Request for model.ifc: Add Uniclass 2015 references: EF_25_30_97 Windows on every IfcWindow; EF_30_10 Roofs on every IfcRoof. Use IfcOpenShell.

First a look at what the model holds.

```python
import ifcopenshell

model = ifcopenshell.open("model.ifc")
print(model.schema)
print("classifications:", [c.Name for c in model.by_type("IfcClassification")])
for ifc_class in ("IfcDoor", "IfcRoof", "IfcStair", "IfcWall", "IfcWindow"):
    print(ifc_class, len(model.by_type(ifc_class)))
```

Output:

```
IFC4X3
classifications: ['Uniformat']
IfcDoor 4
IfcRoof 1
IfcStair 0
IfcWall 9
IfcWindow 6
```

```python
import ifcopenshell
import ifcopenshell.api.classification

model = ifcopenshell.open("model.ifc")

system = ifcopenshell.api.classification.add_classification(model, classification="Uniclass 2015")

codes = {
    "IfcWindow": ("EF_25_30_97", "Windows"),
    "IfcRoof": ("EF_30_10", "Roofs"),
}
for ifc_class, (code, name) in codes.items():
    products = model.by_type(ifc_class)
    ifcopenshell.api.classification.add_reference(
        model, products=products, classification=system, identification=code, name=name
    )
    print(code, len(products))

model.write("model_edited.ifc")
```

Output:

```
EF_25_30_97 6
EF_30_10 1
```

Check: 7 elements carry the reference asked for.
